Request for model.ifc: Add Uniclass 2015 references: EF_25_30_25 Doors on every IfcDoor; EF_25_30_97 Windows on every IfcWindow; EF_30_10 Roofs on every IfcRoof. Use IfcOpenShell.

First a look at what the model holds.

```python
import ifcopenshell

model = ifcopenshell.open("model.ifc")
print(model.schema)
print("classifications:", [c.Name for c in model.by_type("IfcClassification")])
for ifc_class in ("IfcDoor", "IfcRoof", "IfcStair", "IfcWall", "IfcWindow"):
    print(ifc_class, len(model.by_type(ifc_class)))
```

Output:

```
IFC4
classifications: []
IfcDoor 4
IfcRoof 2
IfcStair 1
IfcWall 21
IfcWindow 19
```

```python
import ifcopenshell
import ifcopenshell.api.classification

model = ifcopenshell.open("model.ifc")

system = ifcopenshell.api.classification.add_classification(model, classification="Uniclass 2015")

codes = {
    "IfcDoor": ("EF_25_30_25", "Doors"),
    "IfcWindow": ("EF_25_30_97", "Windows"),
    "IfcRoof": ("EF_30_10", "Roofs"),
}
for ifc_class, (code, name) in codes.items():
    products = model.by_type(ifc_class)
    ifcopenshell.api.classification.add_reference(
        model, products=products, classification=system, identification=code, name=name
    )
    print(code, len(products))

model.write("model_updated.ifc")
```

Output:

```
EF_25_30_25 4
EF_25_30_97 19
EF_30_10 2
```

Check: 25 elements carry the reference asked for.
